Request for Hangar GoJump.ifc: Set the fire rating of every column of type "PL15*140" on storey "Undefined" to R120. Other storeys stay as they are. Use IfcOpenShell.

First a look at what the model holds.

```python
import ifcopenshell
import ifcopenshell.util.element

model = ifcopenshell.open("Hangar GoJump.ifc")
print(model.schema)
storey = next(s for s in model.by_type("IfcBuildingStorey") if s.Name == "Undefined")
columns = [e for e in ifcopenshell.util.element.get_decomposition(storey) if e.is_a("IfcColumn")]
seen = {}
for e in columns:
    element_type = ifcopenshell.util.element.get_type(e)
    key = (element_type.Name if element_type != e and element_type else None, ifcopenshell.util.element.get_pset(e, "Pset_ColumnCommon", "FireRating"))
    seen[key] = seen.get(key, 0) + 1
for (name, value), count in sorted(seen.items(), key=str):
    print(count, "x", name, "|", value)
```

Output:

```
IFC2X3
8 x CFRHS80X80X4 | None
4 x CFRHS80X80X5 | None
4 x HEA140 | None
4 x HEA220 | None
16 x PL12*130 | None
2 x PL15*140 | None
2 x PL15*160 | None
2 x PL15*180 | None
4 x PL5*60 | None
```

```python
import ifcopenshell
import ifcopenshell.api.pset
import ifcopenshell.util.element

model = ifcopenshell.open("Hangar GoJump.ifc")

storey = next(s for s in model.by_type("IfcBuildingStorey") if s.Name == "Undefined")
columns = [e for e in ifcopenshell.util.element.get_decomposition(storey) if e.is_a("IfcColumn")]

count = 0
for e in columns:
    element_type = ifcopenshell.util.element.get_type(e)
    if element_type in (None, e) or element_type.Name != "PL15*140":
        continue
    # add_pset returns the element's existing set when there is one.
    pset = ifcopenshell.api.pset.add_pset(model, product=e, name="Pset_ColumnCommon")
    ifcopenshell.api.pset.edit_pset(model, pset=pset, properties={"FireRating": "R120"})
    count += 1

print(count, "columns updated")

model.write("Hangar GoJump_v2.ifc")
```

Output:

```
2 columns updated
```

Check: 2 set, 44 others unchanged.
